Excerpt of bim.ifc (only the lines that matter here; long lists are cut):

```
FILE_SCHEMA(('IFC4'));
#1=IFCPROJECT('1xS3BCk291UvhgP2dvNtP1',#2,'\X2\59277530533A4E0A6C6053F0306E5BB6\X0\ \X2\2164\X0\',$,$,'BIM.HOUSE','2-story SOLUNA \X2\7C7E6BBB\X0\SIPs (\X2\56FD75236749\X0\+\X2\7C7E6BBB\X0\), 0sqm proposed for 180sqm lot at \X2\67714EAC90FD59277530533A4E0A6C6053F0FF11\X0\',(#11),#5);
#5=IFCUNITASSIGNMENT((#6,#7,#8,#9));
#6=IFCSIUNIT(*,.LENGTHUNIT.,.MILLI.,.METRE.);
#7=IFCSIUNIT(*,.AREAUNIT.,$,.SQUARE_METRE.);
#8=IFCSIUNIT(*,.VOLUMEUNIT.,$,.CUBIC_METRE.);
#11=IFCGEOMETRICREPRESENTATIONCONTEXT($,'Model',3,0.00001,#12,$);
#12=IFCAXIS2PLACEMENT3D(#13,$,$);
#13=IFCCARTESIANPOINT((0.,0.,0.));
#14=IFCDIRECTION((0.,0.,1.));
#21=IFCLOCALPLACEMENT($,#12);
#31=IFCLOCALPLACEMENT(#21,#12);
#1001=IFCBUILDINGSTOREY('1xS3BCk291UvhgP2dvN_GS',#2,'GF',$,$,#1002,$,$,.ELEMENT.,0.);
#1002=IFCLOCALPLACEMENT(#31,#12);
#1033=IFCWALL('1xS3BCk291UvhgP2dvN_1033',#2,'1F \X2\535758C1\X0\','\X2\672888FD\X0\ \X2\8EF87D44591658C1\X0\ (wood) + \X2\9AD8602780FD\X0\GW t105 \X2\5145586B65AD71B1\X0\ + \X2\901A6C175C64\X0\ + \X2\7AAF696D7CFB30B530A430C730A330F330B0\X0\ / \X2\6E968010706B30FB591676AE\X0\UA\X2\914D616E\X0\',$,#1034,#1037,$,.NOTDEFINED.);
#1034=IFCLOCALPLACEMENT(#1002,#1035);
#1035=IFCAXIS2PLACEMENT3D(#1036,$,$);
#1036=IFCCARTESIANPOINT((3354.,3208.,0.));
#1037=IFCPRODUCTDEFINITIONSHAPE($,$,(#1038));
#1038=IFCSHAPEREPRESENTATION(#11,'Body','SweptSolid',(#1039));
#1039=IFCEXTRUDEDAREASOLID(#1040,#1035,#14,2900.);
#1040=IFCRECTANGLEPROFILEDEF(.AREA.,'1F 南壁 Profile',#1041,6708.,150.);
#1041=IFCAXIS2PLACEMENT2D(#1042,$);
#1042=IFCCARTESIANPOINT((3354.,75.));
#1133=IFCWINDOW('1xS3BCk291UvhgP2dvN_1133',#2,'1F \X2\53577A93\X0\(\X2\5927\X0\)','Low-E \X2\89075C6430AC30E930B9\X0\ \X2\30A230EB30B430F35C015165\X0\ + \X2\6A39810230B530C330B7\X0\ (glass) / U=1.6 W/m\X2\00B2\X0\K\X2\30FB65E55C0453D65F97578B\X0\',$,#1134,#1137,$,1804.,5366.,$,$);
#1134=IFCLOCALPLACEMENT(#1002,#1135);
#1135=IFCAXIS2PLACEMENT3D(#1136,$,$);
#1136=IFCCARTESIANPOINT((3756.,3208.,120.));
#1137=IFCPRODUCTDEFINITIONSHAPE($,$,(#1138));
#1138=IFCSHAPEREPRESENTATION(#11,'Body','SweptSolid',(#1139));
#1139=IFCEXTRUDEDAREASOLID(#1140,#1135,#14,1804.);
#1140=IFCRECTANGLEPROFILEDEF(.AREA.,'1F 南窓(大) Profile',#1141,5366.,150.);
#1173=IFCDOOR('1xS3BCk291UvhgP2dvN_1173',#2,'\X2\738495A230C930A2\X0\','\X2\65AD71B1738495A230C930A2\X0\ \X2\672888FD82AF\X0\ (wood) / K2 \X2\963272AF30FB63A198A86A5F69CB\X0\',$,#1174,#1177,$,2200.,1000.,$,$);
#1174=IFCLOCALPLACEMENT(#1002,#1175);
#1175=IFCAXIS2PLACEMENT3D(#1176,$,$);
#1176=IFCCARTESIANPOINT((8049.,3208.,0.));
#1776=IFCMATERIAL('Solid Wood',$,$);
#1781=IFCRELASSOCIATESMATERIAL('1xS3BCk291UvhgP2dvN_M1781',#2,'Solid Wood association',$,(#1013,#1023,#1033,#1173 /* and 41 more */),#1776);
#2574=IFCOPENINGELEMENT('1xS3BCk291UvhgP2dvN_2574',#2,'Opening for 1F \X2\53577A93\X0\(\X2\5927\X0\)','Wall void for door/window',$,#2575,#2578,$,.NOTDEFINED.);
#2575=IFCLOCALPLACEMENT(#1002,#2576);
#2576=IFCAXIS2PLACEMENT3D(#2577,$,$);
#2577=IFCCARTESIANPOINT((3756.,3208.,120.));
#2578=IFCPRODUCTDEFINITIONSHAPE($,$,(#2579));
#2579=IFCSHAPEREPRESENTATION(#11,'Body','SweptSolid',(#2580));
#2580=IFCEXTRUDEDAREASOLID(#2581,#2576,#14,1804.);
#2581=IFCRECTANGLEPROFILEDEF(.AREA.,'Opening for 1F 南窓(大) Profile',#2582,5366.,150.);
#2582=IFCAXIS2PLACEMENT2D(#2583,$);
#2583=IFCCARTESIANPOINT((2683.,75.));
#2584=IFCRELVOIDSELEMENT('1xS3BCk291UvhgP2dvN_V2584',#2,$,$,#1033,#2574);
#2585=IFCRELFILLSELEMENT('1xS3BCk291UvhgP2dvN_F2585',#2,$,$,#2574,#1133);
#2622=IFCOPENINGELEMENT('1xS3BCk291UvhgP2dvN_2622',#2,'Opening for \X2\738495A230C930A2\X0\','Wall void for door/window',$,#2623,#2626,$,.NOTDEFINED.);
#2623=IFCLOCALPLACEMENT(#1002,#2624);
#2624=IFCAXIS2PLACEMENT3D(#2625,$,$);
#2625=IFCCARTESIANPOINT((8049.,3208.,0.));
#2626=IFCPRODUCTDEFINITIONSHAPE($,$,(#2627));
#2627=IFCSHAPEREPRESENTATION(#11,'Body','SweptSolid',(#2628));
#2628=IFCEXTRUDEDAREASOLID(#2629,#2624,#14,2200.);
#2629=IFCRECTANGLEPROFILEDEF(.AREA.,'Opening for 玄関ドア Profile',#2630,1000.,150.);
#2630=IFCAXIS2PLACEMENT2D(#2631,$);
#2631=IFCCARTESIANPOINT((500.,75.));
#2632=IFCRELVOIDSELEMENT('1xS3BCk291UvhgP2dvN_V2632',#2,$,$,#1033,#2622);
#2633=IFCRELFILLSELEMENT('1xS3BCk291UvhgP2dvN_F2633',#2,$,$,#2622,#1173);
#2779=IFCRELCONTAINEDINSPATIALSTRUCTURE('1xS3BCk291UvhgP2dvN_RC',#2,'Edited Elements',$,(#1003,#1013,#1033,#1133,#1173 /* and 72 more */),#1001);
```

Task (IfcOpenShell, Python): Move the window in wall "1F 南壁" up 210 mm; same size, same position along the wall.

```python
import numpy as np
import ifcopenshell
import ifcopenshell.api.geometry
import ifcopenshell.util.placement
import ifcopenshell.util.unit

model = ifcopenshell.open("bim.ifc")
unit_scale = ifcopenshell.util.unit.calculate_unit_scale(model)

window = model.by_id(1133)
opening = window.FillsVoids[0].RelatingOpeningElement
dz = 0.21 / unit_scale

shift = np.array([0.0, 0.0, dz])
# The window is not placed relative to its opening, so move both.
for product in (opening, window):
    matrix = ifcopenshell.util.placement.get_local_placement(product.ObjectPlacement)
    matrix[:3, 3] += shift
    ifcopenshell.api.geometry.edit_object_placement(model, product=product, matrix=matrix, is_si=False)

print(f"moved by {dz * unit_scale:+.3f} m")

model.write("bim_rev.ifc")
```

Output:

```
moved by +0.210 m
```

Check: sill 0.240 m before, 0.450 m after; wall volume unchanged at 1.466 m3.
